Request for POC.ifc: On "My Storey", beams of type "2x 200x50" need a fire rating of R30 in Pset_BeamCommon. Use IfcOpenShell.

First a look at what the model holds.

```python
import ifcopenshell
import ifcopenshell.util.element

model = ifcopenshell.open("POC.ifc")
print(model.schema)
storey = next(s for s in model.by_type("IfcBuildingStorey") if s.Name == "My Storey")
beams = [e for e in ifcopenshell.util.element.get_decomposition(storey) if e.is_a("IfcBeam")]
seen = {}
for e in beams:
    element_type = ifcopenshell.util.element.get_type(e)
    key = (element_type.Name if element_type != e and element_type else None, ifcopenshell.util.element.get_pset(e, "Pset_BeamCommon", "FireRating"))
    seen[key] = seen.get(key, 0) + 1
for (name, value), count in sorted(seen.items(), key=str):
    print(count, "x", name, "|", value)
```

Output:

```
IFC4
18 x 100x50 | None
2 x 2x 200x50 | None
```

```python
import ifcopenshell
import ifcopenshell.api.pset
import ifcopenshell.util.element

model = ifcopenshell.open("POC.ifc")

storey = next(s for s in model.by_type("IfcBuildingStorey") if s.Name == "My Storey")
beams = [e for e in ifcopenshell.util.element.get_decomposition(storey) if e.is_a("IfcBeam")]

count = 0
for e in beams:
    element_type = ifcopenshell.util.element.get_type(e)
    if element_type in (None, e) or element_type.Name != "2x 200x50":
        continue
    # add_pset returns the element's existing set when there is one.
    pset = ifcopenshell.api.pset.add_pset(model, product=e, name="Pset_BeamCommon")
    ifcopenshell.api.pset.edit_pset(model, pset=pset, properties={"FireRating": "R30"})
    count += 1

print(count, "beams updated")

model.write("POC_updated.ifc")
```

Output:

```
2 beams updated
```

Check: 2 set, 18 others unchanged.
